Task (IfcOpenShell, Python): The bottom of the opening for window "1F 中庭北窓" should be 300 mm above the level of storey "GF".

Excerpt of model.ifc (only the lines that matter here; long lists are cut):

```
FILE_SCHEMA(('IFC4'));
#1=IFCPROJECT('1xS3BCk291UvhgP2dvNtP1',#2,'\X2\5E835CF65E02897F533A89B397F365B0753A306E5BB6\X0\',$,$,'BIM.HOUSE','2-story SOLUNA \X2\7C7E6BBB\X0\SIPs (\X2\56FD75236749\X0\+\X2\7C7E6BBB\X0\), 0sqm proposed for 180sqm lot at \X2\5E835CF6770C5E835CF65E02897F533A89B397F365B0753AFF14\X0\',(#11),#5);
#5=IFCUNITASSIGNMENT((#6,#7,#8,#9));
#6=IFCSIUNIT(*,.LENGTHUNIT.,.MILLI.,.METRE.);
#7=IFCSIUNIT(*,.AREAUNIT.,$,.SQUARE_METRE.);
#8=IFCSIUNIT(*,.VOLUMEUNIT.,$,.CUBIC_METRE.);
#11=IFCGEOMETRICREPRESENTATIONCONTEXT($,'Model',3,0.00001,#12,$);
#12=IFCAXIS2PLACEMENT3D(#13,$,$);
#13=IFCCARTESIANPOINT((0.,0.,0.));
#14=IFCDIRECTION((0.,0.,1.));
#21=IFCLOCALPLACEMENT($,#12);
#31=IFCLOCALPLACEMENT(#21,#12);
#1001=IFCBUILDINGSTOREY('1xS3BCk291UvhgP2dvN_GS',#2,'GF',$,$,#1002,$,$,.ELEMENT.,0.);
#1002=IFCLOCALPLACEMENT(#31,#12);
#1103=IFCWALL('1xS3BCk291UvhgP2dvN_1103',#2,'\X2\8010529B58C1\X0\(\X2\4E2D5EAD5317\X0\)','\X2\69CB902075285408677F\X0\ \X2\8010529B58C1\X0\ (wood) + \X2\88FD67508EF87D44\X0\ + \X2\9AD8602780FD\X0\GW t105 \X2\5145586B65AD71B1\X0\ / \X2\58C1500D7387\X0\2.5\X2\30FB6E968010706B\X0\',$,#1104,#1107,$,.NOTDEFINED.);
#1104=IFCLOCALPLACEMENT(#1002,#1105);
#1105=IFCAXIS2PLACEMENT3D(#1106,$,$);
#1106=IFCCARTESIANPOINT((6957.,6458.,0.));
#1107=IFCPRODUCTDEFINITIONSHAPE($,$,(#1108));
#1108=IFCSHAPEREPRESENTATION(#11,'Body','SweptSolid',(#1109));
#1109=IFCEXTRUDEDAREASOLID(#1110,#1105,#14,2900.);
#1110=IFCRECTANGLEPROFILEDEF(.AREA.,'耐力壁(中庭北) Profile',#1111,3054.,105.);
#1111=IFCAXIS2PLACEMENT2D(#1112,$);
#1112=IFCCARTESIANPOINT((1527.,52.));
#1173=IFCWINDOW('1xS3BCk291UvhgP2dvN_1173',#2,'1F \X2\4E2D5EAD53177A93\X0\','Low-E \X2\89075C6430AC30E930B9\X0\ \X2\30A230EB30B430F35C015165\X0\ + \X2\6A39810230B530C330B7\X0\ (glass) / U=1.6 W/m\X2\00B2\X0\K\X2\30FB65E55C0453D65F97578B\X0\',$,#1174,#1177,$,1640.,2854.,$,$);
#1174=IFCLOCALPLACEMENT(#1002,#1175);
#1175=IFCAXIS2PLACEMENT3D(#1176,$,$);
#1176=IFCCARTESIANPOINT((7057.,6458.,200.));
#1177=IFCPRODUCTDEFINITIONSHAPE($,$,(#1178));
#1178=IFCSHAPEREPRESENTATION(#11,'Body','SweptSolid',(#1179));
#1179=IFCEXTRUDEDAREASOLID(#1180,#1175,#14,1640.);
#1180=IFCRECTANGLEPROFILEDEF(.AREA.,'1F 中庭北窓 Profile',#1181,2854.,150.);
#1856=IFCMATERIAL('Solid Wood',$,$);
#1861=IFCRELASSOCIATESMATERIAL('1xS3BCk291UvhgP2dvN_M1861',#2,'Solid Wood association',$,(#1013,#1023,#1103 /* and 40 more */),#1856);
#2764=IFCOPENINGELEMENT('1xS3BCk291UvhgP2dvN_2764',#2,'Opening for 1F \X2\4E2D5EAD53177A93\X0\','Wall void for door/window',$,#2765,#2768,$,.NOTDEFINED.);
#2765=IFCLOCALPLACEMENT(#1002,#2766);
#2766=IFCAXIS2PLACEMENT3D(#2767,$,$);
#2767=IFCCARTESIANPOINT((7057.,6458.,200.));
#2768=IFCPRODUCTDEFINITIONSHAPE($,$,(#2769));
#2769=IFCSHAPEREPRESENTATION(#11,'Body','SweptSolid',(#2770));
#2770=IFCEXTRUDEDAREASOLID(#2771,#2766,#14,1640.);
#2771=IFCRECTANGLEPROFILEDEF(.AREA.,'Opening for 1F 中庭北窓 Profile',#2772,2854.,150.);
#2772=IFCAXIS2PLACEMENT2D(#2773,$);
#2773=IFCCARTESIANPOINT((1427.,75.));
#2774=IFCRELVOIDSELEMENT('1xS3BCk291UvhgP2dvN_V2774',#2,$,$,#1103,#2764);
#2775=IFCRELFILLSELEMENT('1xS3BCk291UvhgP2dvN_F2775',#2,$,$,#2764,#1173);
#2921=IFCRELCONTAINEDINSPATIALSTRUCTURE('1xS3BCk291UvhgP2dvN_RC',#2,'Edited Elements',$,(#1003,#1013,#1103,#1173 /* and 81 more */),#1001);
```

```python
import numpy as np
import ifcopenshell
import ifcopenshell.api.geometry
import ifcopenshell.geom
import ifcopenshell.util.element
import ifcopenshell.util.placement
import ifcopenshell.util.shape
import ifcopenshell.util.unit

model = ifcopenshell.open("model.ifc")
unit_scale = ifcopenshell.util.unit.calculate_unit_scale(model)

window = model.by_id(1173)
opening = window.FillsVoids[0].RelatingOpeningElement
storey = ifcopenshell.util.element.get_container(window, ifc_class="IfcBuildingStorey")
level = ifcopenshell.util.placement.get_local_placement(storey.ObjectPlacement)[2, 3]

# The opening's origin need not be at the sill, so measure its lowest point.
shape = ifcopenshell.geom.create_shape(ifcopenshell.geom.settings(), opening)
bottom = ifcopenshell.util.shape.get_shape_bottom_elevation(shape, shape.geometry) / unit_scale
dz = level + 300.0 - bottom

shift = np.array([0.0, 0.0, dz])
# The window is not placed relative to its opening, so move both.
for product in (opening, window):
    matrix = ifcopenshell.util.placement.get_local_placement(product.ObjectPlacement)
    matrix[:3, 3] += shift
    ifcopenshell.api.geometry.edit_object_placement(model, product=product, matrix=matrix, is_si=False)

print(f"moved by {dz * unit_scale:+.3f} m")

model.write("model_rev.ifc")
```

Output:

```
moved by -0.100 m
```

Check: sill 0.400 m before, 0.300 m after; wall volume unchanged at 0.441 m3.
